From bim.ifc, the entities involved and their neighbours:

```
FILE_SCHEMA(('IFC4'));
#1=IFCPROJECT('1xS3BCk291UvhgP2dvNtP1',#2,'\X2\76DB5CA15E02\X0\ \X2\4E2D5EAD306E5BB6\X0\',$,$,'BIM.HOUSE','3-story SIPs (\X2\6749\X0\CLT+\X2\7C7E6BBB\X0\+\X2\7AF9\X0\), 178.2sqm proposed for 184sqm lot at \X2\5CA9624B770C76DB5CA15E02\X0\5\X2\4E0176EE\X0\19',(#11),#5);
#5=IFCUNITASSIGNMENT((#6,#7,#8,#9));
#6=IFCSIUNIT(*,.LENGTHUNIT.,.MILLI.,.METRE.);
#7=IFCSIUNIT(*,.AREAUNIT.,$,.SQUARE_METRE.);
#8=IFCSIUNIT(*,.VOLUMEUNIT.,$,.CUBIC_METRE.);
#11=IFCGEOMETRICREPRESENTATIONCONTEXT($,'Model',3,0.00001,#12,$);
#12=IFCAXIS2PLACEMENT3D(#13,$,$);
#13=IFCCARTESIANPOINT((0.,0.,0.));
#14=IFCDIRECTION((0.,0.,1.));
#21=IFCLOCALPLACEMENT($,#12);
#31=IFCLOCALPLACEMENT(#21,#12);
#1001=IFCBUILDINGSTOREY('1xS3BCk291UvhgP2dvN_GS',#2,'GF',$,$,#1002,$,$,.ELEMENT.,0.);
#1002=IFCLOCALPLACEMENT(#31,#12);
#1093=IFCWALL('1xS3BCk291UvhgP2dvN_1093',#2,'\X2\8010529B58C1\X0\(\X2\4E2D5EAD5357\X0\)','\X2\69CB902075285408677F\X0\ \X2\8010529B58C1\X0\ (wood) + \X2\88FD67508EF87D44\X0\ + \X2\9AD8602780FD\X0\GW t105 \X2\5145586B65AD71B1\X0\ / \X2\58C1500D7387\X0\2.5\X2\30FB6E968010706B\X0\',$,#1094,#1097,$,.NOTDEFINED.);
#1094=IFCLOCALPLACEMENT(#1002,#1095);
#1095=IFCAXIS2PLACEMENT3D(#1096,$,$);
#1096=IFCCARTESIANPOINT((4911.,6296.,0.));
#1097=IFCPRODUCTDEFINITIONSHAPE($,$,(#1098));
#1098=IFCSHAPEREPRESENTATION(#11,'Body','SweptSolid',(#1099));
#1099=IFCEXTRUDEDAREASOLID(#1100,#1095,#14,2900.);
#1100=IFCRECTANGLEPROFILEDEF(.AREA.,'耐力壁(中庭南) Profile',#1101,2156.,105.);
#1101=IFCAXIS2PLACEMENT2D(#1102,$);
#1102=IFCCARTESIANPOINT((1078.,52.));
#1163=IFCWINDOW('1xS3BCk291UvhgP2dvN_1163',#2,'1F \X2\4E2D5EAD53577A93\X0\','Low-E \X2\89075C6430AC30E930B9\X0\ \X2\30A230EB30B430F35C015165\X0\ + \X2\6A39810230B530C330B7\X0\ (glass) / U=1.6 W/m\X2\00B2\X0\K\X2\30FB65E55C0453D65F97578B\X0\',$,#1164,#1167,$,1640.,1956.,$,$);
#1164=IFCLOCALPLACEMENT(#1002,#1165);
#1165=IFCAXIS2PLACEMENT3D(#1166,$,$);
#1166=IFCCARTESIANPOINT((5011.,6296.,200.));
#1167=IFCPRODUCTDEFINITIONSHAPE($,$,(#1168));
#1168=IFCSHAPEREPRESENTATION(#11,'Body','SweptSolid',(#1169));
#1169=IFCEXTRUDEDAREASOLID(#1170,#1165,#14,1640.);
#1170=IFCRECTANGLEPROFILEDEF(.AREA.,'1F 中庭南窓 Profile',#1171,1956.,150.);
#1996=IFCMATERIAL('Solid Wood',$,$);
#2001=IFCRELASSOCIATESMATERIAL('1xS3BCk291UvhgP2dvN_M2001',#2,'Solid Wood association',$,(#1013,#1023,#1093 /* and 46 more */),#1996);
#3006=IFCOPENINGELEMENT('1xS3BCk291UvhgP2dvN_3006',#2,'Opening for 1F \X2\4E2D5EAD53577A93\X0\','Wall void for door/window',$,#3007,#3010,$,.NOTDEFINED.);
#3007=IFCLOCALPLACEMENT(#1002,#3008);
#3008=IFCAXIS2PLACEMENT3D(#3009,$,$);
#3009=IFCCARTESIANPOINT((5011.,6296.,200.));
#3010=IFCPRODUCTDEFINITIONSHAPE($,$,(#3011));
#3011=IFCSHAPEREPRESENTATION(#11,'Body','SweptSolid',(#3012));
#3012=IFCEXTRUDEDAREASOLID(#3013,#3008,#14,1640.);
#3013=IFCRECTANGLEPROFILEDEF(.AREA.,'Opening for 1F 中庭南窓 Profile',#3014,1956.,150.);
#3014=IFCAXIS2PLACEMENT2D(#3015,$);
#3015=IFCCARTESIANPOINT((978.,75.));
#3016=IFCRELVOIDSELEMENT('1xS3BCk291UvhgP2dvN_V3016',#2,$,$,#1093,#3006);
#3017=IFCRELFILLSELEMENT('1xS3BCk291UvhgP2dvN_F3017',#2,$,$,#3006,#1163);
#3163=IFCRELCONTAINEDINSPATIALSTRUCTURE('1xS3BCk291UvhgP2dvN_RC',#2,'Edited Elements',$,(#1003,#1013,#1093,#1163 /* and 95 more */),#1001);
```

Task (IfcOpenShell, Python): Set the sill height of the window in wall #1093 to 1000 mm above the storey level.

```python
import numpy as np
import ifcopenshell
import ifcopenshell.api.geometry
import ifcopenshell.geom
import ifcopenshell.util.element
import ifcopenshell.util.placement
import ifcopenshell.util.shape
import ifcopenshell.util.unit

model = ifcopenshell.open("bim.ifc")
unit_scale = ifcopenshell.util.unit.calculate_unit_scale(model)

window = model.by_guid("1xS3BCk291UvhgP2dvN_1163")
opening = window.FillsVoids[0].RelatingOpeningElement
storey = ifcopenshell.util.element.get_container(window, ifc_class="IfcBuildingStorey")
level = ifcopenshell.util.placement.get_local_placement(storey.ObjectPlacement)[2, 3]

# The opening's origin need not be at the sill, so measure its lowest point.
shape = ifcopenshell.geom.create_shape(ifcopenshell.geom.settings(), opening)
bottom = ifcopenshell.util.shape.get_shape_bottom_elevation(shape, shape.geometry) / unit_scale
dz = level + 1 / unit_scale - bottom

shift = np.array([0.0, 0.0, dz])
# The window is not placed relative to its opening, so move both.
for product in (opening, window):
    matrix = ifcopenshell.util.placement.get_local_placement(product.ObjectPlacement)
    matrix[:3, 3] += shift
    ifcopenshell.api.geometry.edit_object_placement(model, product=product, matrix=matrix, is_si=False)

print(f"moved by {dz * unit_scale:+.3f} m")

model.write("bim_edited.ifc")
```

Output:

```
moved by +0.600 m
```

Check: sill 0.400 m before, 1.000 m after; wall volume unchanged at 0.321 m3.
